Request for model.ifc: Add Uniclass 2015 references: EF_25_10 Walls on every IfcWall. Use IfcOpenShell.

First a look at what the model holds.

```python
import ifcopenshell

model = ifcopenshell.open("model.ifc")
print(model.schema)
print("classifications:", [c.Name for c in model.by_type("IfcClassification")])
for ifc_class in ("IfcDoor", "IfcRoof", "IfcStair", "IfcWall", "IfcWindow"):
    print(ifc_class, len(model.by_type(ifc_class)))
```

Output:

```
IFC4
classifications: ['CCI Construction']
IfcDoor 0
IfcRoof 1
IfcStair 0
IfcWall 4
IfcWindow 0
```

```python
import ifcopenshell
import ifcopenshell.api.classification

model = ifcopenshell.open("model.ifc")

system = ifcopenshell.api.classification.add_classification(model, classification="Uniclass 2015")

codes = {
    "IfcWall": ("EF_25_10", "Walls"),
}
for ifc_class, (code, name) in codes.items():
    products = model.by_type(ifc_class)
    ifcopenshell.api.classification.add_reference(
        model, products=products, classification=system, identification=code, name=name
    )
    print(code, len(products))

model.write("model_v2.ifc")
```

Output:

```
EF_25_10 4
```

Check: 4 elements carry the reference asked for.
